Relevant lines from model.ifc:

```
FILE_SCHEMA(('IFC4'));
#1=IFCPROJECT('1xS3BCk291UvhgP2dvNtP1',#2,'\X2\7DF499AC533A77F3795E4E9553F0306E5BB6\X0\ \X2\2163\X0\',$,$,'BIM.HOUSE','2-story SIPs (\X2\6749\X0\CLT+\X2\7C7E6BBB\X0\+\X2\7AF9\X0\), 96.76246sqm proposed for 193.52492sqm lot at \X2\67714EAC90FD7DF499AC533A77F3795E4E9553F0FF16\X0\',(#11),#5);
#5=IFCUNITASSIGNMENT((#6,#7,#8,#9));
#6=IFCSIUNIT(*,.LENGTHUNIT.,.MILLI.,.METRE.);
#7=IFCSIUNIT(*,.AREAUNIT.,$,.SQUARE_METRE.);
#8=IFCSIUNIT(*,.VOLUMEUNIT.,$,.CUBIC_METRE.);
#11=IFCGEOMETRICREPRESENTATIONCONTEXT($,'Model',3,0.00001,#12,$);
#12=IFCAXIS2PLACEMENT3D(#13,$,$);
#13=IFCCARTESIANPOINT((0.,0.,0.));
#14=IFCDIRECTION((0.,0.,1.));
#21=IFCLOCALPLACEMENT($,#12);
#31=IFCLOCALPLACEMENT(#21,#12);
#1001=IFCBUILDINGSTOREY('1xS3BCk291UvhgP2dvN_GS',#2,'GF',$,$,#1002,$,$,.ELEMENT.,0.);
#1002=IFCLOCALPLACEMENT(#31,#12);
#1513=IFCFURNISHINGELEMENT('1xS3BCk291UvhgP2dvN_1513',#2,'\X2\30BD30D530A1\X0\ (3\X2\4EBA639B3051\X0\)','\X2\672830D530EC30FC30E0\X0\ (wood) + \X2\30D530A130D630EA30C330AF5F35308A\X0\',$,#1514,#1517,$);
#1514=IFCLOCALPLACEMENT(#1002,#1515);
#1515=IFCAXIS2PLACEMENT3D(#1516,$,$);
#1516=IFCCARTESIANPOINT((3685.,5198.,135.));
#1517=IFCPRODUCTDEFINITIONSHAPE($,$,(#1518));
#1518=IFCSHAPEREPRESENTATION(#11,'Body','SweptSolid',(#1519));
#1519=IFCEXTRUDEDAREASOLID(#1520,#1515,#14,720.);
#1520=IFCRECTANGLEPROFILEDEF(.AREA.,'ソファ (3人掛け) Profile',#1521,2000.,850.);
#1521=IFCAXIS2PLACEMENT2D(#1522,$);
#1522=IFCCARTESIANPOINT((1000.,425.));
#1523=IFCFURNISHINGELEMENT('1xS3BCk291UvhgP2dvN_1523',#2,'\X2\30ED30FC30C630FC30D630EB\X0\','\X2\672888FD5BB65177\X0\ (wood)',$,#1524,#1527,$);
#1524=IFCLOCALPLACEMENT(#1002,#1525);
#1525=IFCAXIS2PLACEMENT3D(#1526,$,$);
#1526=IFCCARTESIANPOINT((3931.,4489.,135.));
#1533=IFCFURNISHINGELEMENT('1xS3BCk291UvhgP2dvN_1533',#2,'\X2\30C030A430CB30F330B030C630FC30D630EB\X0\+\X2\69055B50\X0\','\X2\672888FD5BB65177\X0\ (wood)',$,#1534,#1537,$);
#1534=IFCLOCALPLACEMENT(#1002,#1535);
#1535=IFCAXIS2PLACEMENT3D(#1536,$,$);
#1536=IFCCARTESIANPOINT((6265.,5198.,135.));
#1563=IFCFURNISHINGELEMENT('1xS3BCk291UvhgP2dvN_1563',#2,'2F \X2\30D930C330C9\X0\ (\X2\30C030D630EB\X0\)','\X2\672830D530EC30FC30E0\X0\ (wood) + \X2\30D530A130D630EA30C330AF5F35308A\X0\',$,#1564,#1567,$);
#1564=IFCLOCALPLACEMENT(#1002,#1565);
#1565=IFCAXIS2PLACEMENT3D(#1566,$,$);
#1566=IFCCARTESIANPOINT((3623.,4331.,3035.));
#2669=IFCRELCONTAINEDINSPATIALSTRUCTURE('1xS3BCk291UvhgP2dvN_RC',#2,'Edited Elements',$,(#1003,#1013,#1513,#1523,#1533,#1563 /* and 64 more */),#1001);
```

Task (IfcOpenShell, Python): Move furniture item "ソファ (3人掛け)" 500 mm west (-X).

```python
import ifcopenshell
import ifcopenshell.api.geometry
import ifcopenshell.util.placement
import ifcopenshell.util.unit

model = ifcopenshell.open("model.ifc")
unit_scale = ifcopenshell.util.unit.calculate_unit_scale(model)

item = model.by_guid("1xS3BCk291UvhgP2dvN_1513")
matrix = ifcopenshell.util.placement.get_local_placement(item.ObjectPlacement)
matrix[0, 3] -= 0.5 / unit_scale
ifcopenshell.api.geometry.edit_object_placement(model, product=item, matrix=matrix, is_si=False)

print(ifcopenshell.util.placement.get_local_placement(item.ObjectPlacement).round(3) + 0.0)

model.write("model_updated.ifc")
```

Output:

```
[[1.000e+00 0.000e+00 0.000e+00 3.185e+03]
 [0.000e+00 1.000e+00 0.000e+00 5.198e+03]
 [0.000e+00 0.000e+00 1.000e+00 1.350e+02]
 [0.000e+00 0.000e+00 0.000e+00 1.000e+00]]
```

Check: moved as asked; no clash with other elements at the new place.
